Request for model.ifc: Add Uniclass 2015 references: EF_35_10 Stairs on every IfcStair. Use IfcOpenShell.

First a look at what the model holds.

```python
import ifcopenshell

model = ifcopenshell.open("model.ifc")
print(model.schema)
print("classifications:", [c.Name for c in model.by_type("IfcClassification")])
for ifc_class in ("IfcDoor", "IfcRoof", "IfcStair", "IfcWall", "IfcWindow"):
    print(ifc_class, len(model.by_type(ifc_class)))
```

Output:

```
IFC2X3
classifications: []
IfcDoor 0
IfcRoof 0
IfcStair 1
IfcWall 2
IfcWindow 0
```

```python
import ifcopenshell
import ifcopenshell.api.classification

model = ifcopenshell.open("model.ifc")

# IFC2X3 requires Source and Edition and has no link from the project to the system.
system = model.create_entity("IfcClassification", Source="NBS", Edition="2015", Name="Uniclass 2015")

codes = {
    "IfcStair": ("EF_35_10", "Stairs"),
}
for ifc_class, (code, name) in codes.items():
    products = model.by_type(ifc_class)
    ifcopenshell.api.classification.add_reference(
        model, products=products, classification=system, identification=code, name=name
    )
    print(code, len(products))

model.write("model_rev.ifc")
```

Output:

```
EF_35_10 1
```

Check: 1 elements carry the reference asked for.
